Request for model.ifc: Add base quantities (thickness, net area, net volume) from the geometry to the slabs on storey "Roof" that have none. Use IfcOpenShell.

First a look at what the model holds.

```python
import ifcopenshell
import ifcopenshell.util.element
import ifcopenshell.util.unit

model = ifcopenshell.open("model.ifc")
print(model.schema)
for unit_type in ("LENGTHUNIT", "AREAUNIT", "VOLUMEUNIT"):
    print(unit_type, ifcopenshell.util.unit.calculate_unit_scale(model, unit_type))
storey = next(s for s in model.by_type("IfcBuildingStorey") if s.Name == "Roof")
slabs = [e for e in ifcopenshell.util.element.get_decomposition(storey) if e.is_a("IfcSlab")]
for e in sorted(slabs, key=lambda e: e.id()):
    print(e.id(), e.is_a(), e.Name, list(ifcopenshell.util.element.get_psets(e, qtos_only=True)), sep=" | ")
```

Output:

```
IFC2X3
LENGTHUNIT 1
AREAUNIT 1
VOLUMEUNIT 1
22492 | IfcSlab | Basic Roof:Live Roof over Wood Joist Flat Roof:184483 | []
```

```python
import ifcopenshell
import ifcopenshell.api.pset
import ifcopenshell.geom
import ifcopenshell.util.element
import ifcopenshell.util.shape
import ifcopenshell.util.unit

model = ifcopenshell.open("model.ifc")
unit_scale = ifcopenshell.util.unit.calculate_unit_scale(model)
area_scale = ifcopenshell.util.unit.calculate_unit_scale(model, "AREAUNIT")
volume_scale = ifcopenshell.util.unit.calculate_unit_scale(model, "VOLUMEUNIT")
settings = ifcopenshell.geom.settings()

storey = next(s for s in model.by_type("IfcBuildingStorey") if s.Name == "Roof")
slabs = [e for e in ifcopenshell.util.element.get_decomposition(storey) if e.is_a("IfcSlab")]

for e in sorted(slabs, key=lambda e: e.id()):
    if ifcopenshell.util.element.get_psets(e, qtos_only=True, should_inherit=False):
        continue
    # Geometry comes back in metres, in the element's own axes.
    shape = ifcopenshell.geom.create_shape(settings, e)
    values = {
        "Width": ifcopenshell.util.shape.get_z(shape.geometry) / unit_scale,
        "NetArea": ifcopenshell.util.shape.get_footprint_area(shape.geometry) / area_scale,
        "NetVolume": ifcopenshell.util.shape.get_volume(shape.geometry) / volume_scale,
    }
    qto = ifcopenshell.api.pset.add_qto(model, product=e, name="BaseQuantities")
    ifcopenshell.api.pset.edit_qto(model, qto=qto, properties=values)
    print(e.id(), {k: round(v, 3) for k, v in values.items()})

model.write("model_edited.ifc")
```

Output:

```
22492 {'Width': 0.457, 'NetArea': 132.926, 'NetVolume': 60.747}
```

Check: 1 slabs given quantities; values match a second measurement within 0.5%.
